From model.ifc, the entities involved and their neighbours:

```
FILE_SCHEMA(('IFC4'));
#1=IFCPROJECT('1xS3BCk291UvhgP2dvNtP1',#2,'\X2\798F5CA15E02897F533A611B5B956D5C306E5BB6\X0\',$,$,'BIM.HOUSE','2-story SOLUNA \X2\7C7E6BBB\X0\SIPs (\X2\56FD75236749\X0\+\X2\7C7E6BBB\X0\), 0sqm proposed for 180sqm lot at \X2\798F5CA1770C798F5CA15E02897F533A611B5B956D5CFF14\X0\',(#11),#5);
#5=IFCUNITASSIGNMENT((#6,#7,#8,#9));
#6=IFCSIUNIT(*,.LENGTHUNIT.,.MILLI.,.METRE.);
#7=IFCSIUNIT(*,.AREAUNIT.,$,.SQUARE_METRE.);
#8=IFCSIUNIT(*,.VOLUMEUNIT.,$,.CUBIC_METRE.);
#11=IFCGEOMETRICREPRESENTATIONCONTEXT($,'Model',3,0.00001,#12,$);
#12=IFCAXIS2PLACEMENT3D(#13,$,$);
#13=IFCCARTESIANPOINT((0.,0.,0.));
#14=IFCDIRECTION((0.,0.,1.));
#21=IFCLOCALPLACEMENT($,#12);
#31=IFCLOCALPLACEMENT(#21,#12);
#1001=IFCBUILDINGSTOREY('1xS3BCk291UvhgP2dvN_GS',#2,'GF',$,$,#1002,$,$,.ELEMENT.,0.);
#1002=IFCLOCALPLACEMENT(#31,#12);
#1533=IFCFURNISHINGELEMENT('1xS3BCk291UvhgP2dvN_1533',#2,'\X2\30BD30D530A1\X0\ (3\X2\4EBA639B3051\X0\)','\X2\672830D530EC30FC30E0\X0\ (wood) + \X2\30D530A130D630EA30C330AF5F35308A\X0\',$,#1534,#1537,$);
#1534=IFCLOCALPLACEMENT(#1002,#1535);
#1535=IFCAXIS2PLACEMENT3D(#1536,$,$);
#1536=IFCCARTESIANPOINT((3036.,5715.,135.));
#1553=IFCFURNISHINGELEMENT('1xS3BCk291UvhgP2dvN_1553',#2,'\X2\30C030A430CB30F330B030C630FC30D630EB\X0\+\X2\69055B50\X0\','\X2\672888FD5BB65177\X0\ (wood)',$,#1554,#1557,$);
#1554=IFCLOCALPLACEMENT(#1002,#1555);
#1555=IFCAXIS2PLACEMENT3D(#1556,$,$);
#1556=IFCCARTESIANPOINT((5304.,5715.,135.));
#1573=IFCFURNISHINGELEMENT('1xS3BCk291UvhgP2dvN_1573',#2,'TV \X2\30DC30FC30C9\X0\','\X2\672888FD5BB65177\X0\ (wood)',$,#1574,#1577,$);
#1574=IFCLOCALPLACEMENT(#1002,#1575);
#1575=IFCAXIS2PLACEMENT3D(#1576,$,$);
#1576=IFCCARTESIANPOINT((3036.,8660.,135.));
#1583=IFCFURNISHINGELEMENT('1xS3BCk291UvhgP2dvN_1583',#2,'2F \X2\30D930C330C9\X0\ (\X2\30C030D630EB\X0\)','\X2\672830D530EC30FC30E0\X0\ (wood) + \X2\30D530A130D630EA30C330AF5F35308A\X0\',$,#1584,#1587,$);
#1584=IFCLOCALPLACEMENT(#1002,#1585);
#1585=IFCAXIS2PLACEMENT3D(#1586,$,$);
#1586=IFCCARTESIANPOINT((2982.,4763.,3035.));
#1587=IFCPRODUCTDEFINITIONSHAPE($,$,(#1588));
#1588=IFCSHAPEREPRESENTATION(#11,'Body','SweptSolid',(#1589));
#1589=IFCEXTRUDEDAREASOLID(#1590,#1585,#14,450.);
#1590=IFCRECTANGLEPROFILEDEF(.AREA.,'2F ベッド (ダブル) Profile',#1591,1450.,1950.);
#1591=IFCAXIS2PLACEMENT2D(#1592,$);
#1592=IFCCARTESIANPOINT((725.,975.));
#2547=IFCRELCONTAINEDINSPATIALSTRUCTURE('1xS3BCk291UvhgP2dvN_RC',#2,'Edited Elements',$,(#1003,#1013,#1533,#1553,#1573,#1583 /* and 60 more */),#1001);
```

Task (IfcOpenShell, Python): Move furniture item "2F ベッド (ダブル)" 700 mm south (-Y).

```python
import ifcopenshell
import ifcopenshell.api.geometry
import ifcopenshell.util.placement
import ifcopenshell.util.unit

model = ifcopenshell.open("model.ifc")
unit_scale = ifcopenshell.util.unit.calculate_unit_scale(model)

item = model.by_id(1583)
matrix = ifcopenshell.util.placement.get_local_placement(item.ObjectPlacement)
matrix[1, 3] -= 0.7 / unit_scale
ifcopenshell.api.geometry.edit_object_placement(model, product=item, matrix=matrix, is_si=False)

print(ifcopenshell.util.placement.get_local_placement(item.ObjectPlacement).round(3) + 0.0)

model.write("model_updated.ifc")
```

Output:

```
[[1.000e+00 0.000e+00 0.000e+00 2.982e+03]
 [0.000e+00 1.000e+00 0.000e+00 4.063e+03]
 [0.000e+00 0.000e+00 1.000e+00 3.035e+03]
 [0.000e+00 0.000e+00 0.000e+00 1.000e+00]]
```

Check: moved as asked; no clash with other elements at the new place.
